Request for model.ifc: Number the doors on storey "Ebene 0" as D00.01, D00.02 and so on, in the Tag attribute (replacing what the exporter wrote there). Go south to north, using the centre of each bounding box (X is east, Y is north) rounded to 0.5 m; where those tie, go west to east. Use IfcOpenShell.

First a look at what the model holds.

```python
import ifcopenshell
import ifcopenshell.util.element
import ifcopenshell.util.placement

model = ifcopenshell.open("model.ifc")
print(model.schema)
storey = next(s for s in model.by_type("IfcBuildingStorey") if s.Name == "Ebene 0")
doors = [e for e in ifcopenshell.util.element.get_decomposition(storey) if e.is_a("IfcDoor")]
for e in sorted(doors, key=lambda e: e.id()):
    origin = ifcopenshell.util.placement.get_local_placement(e.ObjectPlacement)[:3, 3]
    print(e.id(), e.Tag, e.Name, origin.round(2) + 0.0, sep=" | ")
```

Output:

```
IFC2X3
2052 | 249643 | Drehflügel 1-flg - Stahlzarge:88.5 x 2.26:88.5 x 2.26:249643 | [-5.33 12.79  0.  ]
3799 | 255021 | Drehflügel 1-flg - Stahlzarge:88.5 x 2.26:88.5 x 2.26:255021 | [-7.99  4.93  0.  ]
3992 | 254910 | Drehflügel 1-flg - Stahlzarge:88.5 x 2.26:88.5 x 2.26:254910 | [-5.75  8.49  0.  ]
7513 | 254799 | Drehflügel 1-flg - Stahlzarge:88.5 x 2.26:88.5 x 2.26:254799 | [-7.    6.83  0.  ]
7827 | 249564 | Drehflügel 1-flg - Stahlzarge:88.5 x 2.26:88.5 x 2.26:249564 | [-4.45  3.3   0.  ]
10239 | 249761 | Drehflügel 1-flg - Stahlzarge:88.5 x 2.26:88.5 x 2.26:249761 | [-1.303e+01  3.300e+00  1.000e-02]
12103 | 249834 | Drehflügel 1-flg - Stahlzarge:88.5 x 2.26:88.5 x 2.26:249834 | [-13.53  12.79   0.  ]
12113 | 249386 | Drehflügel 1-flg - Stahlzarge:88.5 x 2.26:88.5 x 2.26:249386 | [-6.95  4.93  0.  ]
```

```python
import ifcopenshell
import ifcopenshell.geom
import ifcopenshell.util.element
import ifcopenshell.util.shape

model = ifcopenshell.open("model.ifc")
settings = ifcopenshell.geom.settings()
settings.set("use-world-coords", True)


def centre(element):
    shape = ifcopenshell.geom.create_shape(settings, element)
    return ifcopenshell.util.shape.get_bbox_centroid(shape.geometry)


storey = next(s for s in model.by_type("IfcBuildingStorey") if s.Name == "Ebene 0")
doors = [e for e in ifcopenshell.util.element.get_decomposition(storey) if e.is_a("IfcDoor")]

# Insertion points can sit at a corner or the storey origin, so sort by the geometry (in metres).
centres = {e: centre(e) for e in doors}
doors.sort(key=lambda e: (round(centres[e][1] / 0.5), centres[e][0]))

for i, e in enumerate(doors, start=1):
    number = f"D00.{i:02d}"
    e.Tag = number
    print(e.id(), number)

model.write("model_edited.ifc")
```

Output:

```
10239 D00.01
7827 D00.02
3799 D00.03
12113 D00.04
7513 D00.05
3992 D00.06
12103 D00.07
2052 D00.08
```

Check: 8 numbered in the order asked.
